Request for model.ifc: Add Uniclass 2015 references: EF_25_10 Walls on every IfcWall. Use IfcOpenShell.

First a look at what the model holds.

```python
import ifcopenshell

model = ifcopenshell.open("model.ifc")
print(model.schema)
print("classifications:", [c.Name for c in model.by_type("IfcClassification")])
for ifc_class in ("IfcDoor", "IfcRoof", "IfcStair", "IfcWall", "IfcWindow"):
    print(ifc_class, len(model.by_type(ifc_class)))
```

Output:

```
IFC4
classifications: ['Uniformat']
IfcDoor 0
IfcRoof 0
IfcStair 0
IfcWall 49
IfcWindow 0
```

```python
import ifcopenshell
import ifcopenshell.api.classification

model = ifcopenshell.open("model.ifc")

system = ifcopenshell.api.classification.add_classification(model, classification="Uniclass 2015")

codes = {
    "IfcWall": ("EF_25_10", "Walls"),
}
for ifc_class, (code, name) in codes.items():
    products = model.by_type(ifc_class)
    ifcopenshell.api.classification.add_reference(
        model, products=products, classification=system, identification=code, name=name
    )
    print(code, len(products))

model.write("model_edited.ifc")
```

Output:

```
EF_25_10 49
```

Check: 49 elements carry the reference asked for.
